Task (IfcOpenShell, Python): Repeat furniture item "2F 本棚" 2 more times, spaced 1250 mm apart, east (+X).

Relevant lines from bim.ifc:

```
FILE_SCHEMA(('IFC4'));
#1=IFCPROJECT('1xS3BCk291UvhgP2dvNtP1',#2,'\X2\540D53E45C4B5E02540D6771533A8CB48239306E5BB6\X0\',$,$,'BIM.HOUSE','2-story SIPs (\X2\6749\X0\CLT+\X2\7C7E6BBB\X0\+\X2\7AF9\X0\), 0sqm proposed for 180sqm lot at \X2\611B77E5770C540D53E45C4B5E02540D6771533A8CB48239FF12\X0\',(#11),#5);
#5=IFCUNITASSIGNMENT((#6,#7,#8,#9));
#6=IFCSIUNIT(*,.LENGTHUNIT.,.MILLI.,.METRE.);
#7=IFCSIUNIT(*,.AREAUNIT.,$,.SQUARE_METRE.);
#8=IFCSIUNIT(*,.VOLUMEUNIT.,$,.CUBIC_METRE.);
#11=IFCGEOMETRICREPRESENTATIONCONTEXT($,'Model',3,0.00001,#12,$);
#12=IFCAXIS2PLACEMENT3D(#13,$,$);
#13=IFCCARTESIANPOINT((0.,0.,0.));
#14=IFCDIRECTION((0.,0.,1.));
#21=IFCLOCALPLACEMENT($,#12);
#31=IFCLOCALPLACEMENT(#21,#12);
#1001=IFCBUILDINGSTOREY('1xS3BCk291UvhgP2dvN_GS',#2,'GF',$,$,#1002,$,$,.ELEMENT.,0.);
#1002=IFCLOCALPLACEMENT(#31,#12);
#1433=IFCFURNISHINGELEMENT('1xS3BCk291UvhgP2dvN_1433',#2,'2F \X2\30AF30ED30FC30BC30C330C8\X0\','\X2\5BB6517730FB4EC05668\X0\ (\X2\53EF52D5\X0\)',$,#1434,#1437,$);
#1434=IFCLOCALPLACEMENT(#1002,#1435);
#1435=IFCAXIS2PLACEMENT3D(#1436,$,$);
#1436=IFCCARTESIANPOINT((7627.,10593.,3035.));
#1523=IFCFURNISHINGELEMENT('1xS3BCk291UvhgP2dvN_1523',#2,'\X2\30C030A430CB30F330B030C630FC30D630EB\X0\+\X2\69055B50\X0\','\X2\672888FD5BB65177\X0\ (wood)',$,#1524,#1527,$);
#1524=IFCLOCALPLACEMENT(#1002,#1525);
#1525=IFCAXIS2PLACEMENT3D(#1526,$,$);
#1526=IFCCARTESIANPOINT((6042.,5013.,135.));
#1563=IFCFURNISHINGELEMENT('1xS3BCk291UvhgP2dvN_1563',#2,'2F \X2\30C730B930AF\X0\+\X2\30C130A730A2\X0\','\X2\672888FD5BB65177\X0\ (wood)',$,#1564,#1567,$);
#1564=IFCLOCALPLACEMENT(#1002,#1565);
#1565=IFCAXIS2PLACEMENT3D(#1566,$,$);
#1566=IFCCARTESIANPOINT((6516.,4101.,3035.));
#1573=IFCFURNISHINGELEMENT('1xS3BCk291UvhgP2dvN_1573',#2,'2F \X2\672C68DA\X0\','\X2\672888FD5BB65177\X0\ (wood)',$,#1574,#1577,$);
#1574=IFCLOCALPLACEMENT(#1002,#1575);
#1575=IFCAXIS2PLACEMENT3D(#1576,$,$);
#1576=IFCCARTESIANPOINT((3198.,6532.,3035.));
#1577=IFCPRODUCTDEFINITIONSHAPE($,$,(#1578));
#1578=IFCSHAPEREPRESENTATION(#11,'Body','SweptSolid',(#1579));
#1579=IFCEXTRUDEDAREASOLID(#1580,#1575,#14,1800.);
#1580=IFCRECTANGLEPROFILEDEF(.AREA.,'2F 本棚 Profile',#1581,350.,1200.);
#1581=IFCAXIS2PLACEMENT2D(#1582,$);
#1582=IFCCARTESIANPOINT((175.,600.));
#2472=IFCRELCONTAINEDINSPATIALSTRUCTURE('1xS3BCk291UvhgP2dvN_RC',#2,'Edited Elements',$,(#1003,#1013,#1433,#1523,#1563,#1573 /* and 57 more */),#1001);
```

```python
import numpy as np
import ifcopenshell
import ifcopenshell.api.geometry
import ifcopenshell.api.root
import ifcopenshell.util.element
import ifcopenshell.util.placement

model = ifcopenshell.open("bim.ifc")


def reuse_history(source, copy):
    """copy_class also copies each property set's owner history, people and application; keep the originals."""
    for rel in copy.IsDefinedBy:
        if rel.is_a("IfcRelDefinesByProperties") and (history := rel.RelatingPropertyDefinition.OwnerHistory):
            rel.RelatingPropertyDefinition.OwnerHistory = source.OwnerHistory
            ifcopenshell.util.element.remove_deep2(model, history)


source = model.by_guid("1xS3BCk291UvhgP2dvN_1573")
base = ifcopenshell.util.placement.get_local_placement(source.ObjectPlacement)
step = np.array([1.0, 0.0, 0.0]) * 1250.0

for i in range(1, 3):
    copy = ifcopenshell.api.root.copy_class(model, product=source)
    copy.Representation = ifcopenshell.util.element.copy_deep(
        model, source.Representation, exclude=["IfcGeometricRepresentationContext", "IfcRepresentationMap"]
    )
    reuse_history(source, copy)
    matrix = base.copy()
    matrix[:3, 3] += i * step
    print("added at", matrix[:3, 3].round(3) + 0.0)
    ifcopenshell.api.geometry.edit_object_placement(model, product=copy, matrix=matrix, is_si=False)

model.write("bim_v2.ifc")
```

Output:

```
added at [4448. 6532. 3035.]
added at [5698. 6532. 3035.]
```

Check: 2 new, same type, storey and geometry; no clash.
